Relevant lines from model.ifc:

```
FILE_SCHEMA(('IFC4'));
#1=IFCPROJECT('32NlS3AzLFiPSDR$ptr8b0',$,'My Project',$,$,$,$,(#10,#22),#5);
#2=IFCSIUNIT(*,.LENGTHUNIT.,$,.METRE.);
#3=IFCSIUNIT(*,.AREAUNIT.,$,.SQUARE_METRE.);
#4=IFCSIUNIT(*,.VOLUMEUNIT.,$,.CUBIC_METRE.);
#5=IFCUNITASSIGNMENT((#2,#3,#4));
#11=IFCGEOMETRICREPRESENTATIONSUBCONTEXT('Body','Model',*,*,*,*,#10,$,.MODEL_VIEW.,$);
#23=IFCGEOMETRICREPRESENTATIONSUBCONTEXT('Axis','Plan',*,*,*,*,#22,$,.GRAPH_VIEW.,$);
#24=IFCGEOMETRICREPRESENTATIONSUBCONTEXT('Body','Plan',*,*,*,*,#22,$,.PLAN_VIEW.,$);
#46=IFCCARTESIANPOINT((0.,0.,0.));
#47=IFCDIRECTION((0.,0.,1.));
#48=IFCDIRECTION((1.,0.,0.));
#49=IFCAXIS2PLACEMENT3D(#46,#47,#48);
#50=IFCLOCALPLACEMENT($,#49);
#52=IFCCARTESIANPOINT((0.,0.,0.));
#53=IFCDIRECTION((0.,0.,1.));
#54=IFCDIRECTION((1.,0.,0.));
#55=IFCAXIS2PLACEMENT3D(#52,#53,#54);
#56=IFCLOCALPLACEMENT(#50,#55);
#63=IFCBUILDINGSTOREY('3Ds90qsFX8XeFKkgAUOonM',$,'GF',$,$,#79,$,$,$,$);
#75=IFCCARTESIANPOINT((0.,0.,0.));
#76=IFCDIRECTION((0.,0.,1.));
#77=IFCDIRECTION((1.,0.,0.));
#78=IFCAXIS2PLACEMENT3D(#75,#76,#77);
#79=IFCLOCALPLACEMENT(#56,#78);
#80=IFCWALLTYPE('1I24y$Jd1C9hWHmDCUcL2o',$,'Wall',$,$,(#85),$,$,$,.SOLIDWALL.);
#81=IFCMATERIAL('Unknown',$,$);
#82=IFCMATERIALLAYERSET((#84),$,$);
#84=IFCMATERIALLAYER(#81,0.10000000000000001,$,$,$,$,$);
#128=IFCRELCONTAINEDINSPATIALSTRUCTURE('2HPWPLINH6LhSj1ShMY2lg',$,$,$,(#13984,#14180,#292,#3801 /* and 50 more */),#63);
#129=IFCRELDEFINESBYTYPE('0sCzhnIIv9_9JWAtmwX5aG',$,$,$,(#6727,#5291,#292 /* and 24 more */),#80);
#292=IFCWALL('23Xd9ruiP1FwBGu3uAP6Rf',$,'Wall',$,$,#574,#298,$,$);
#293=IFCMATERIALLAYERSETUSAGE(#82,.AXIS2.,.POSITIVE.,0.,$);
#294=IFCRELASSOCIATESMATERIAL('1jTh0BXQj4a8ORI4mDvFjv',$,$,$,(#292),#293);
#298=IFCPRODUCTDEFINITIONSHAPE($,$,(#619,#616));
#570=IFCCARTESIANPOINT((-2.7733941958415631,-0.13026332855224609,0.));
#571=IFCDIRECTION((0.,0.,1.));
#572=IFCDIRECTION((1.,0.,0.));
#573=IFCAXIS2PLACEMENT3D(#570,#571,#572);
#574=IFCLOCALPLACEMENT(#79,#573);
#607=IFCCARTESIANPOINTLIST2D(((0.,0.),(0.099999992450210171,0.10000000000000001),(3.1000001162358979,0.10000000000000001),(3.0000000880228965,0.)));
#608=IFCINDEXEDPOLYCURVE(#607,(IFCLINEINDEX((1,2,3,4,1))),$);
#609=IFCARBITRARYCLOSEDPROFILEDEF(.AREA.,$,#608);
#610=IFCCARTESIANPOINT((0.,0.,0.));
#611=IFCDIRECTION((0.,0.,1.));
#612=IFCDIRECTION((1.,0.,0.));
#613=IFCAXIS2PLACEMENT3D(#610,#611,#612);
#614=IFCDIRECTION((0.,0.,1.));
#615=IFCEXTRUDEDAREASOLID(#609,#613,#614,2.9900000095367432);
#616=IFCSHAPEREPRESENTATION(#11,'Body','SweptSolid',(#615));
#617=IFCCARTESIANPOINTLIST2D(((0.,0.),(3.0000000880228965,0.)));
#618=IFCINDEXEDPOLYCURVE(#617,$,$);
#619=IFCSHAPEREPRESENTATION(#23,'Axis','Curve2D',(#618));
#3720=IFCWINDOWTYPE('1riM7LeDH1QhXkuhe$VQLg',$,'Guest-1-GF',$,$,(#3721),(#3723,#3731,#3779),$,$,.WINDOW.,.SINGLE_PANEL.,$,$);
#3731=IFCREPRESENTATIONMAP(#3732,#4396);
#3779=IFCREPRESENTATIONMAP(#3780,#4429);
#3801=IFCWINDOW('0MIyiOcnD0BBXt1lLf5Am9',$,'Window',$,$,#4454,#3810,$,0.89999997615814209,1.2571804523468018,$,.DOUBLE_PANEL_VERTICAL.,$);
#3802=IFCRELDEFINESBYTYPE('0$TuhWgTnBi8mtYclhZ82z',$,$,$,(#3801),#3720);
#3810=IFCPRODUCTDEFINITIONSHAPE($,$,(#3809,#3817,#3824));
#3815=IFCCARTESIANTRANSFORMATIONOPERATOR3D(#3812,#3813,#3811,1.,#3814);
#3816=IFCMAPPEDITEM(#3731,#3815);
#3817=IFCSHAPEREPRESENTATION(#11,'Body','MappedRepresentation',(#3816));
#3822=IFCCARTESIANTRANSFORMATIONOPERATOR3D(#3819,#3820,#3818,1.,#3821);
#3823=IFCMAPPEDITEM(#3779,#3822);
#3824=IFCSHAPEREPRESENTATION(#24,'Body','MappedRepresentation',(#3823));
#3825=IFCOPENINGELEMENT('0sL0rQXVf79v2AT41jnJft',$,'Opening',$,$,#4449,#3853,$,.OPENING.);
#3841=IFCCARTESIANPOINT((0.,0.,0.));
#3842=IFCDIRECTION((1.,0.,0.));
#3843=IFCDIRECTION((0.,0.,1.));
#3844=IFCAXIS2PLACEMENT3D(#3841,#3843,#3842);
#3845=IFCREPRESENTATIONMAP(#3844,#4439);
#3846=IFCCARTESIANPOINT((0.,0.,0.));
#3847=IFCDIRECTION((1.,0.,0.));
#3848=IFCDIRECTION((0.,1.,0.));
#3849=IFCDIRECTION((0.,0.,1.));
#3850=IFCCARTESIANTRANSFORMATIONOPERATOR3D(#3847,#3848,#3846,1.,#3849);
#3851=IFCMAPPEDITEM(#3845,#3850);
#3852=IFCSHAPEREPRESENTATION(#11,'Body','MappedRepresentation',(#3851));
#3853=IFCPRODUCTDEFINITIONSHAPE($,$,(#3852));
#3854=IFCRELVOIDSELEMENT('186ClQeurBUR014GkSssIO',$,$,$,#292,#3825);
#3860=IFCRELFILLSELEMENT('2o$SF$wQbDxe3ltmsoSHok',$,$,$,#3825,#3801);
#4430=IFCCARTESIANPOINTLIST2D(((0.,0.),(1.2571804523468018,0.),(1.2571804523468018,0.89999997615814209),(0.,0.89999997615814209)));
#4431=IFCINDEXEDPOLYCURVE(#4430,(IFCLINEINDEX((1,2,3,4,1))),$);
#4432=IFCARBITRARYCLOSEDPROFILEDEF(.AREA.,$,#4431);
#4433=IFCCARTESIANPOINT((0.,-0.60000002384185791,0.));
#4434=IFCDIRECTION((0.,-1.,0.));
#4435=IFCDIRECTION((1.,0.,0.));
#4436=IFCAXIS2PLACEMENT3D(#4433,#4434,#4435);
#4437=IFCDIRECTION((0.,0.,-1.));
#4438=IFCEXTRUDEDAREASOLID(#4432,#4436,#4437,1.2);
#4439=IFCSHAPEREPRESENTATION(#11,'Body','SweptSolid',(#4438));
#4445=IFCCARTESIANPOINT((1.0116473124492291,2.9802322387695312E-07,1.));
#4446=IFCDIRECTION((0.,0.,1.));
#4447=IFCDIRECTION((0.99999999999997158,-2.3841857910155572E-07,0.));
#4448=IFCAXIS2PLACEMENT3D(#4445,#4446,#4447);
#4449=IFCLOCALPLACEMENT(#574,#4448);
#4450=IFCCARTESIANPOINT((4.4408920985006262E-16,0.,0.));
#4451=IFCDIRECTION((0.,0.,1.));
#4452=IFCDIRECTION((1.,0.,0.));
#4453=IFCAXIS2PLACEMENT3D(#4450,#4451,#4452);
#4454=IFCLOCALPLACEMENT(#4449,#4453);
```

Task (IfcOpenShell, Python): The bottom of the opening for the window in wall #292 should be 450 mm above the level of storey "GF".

```python
import numpy as np
import ifcopenshell
import ifcopenshell.api.geometry
import ifcopenshell.geom
import ifcopenshell.util.element
import ifcopenshell.util.placement
import ifcopenshell.util.shape
import ifcopenshell.util.unit

model = ifcopenshell.open("model.ifc")
unit_scale = ifcopenshell.util.unit.calculate_unit_scale(model)

window = model.by_guid("0MIyiOcnD0BBXt1lLf5Am9")
opening = window.FillsVoids[0].RelatingOpeningElement
storey = ifcopenshell.util.element.get_container(window, ifc_class="IfcBuildingStorey")
level = ifcopenshell.util.placement.get_local_placement(storey.ObjectPlacement)[2, 3]

# The opening's origin need not be at the sill, so measure its lowest point.
shape = ifcopenshell.geom.create_shape(ifcopenshell.geom.settings(), opening)
bottom = ifcopenshell.util.shape.get_shape_bottom_elevation(shape, shape.geometry) / unit_scale
dz = level + 0.45 - bottom

shift = np.array([0.0, 0.0, dz])
# The window is placed relative to its opening, so it follows when the opening moves.
matrix = ifcopenshell.util.placement.get_local_placement(opening.ObjectPlacement)
matrix[:3, 3] += shift
ifcopenshell.api.geometry.edit_object_placement(
    model, product=opening, matrix=matrix, is_si=False, should_transform_children=True
)

print(f"moved by {dz * unit_scale:+.3f} m")

model.write("model_edited.ifc")
```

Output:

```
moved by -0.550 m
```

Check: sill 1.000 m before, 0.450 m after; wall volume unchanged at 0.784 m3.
